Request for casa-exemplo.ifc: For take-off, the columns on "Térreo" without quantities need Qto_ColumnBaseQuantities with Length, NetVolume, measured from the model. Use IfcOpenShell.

First a look at what the model holds.

```python
import ifcopenshell
import ifcopenshell.util.element
import ifcopenshell.util.unit

model = ifcopenshell.open("casa-exemplo.ifc")
print(model.schema)
for unit_type in ("LENGTHUNIT", "AREAUNIT", "VOLUMEUNIT"):
    print(unit_type, ifcopenshell.util.unit.calculate_unit_scale(model, unit_type))
storey = next(s for s in model.by_type("IfcBuildingStorey") if s.Name == "Térreo")
columns = [e for e in ifcopenshell.util.element.get_decomposition(storey) if e.is_a("IfcColumn")]
for e in sorted(columns, key=lambda e: e.id()):
    print(e.id(), e.is_a(), e.Name, list(ifcopenshell.util.element.get_psets(e, qtos_only=True)), sep=" | ")
```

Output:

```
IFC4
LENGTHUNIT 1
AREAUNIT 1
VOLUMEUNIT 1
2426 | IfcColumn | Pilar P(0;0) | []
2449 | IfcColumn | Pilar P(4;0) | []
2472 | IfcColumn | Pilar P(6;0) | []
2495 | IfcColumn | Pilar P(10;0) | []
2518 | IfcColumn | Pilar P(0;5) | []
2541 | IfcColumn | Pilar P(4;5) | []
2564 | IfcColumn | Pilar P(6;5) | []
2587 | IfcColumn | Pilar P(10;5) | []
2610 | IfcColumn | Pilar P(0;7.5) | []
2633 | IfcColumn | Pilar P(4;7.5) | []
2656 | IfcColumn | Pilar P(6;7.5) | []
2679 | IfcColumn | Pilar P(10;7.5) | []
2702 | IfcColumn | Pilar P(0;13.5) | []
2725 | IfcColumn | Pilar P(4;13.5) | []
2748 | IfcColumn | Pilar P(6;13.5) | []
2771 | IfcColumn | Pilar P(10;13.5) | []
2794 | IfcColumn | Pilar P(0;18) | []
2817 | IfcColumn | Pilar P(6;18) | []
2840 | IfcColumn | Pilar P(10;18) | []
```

```python
import ifcopenshell
import ifcopenshell.api.pset
import ifcopenshell.geom
import ifcopenshell.util.element
import ifcopenshell.util.shape
import ifcopenshell.util.unit

model = ifcopenshell.open("casa-exemplo.ifc")
unit_scale = ifcopenshell.util.unit.calculate_unit_scale(model)
volume_scale = ifcopenshell.util.unit.calculate_unit_scale(model, "VOLUMEUNIT")
settings = ifcopenshell.geom.settings()

storey = next(s for s in model.by_type("IfcBuildingStorey") if s.Name == "Térreo")
columns = [e for e in ifcopenshell.util.element.get_decomposition(storey) if e.is_a("IfcColumn")]

for e in sorted(columns, key=lambda e: e.id()):
    if ifcopenshell.util.element.get_psets(e, qtos_only=True, should_inherit=False):
        continue
    # Geometry comes back in metres, in the element's own axes.
    shape = ifcopenshell.geom.create_shape(settings, e)
    values = {
        "Length": ifcopenshell.util.shape.get_z(shape.geometry) / unit_scale,
        "NetVolume": ifcopenshell.util.shape.get_volume(shape.geometry) / volume_scale,
    }
    qto = ifcopenshell.api.pset.add_qto(model, product=e, name="Qto_ColumnBaseQuantities")
    ifcopenshell.api.pset.edit_qto(model, qto=qto, properties=values)
    print(e.id(), {k: round(v, 3) for k, v in values.items()})

model.write("casa-exemplo_v2.ifc")
```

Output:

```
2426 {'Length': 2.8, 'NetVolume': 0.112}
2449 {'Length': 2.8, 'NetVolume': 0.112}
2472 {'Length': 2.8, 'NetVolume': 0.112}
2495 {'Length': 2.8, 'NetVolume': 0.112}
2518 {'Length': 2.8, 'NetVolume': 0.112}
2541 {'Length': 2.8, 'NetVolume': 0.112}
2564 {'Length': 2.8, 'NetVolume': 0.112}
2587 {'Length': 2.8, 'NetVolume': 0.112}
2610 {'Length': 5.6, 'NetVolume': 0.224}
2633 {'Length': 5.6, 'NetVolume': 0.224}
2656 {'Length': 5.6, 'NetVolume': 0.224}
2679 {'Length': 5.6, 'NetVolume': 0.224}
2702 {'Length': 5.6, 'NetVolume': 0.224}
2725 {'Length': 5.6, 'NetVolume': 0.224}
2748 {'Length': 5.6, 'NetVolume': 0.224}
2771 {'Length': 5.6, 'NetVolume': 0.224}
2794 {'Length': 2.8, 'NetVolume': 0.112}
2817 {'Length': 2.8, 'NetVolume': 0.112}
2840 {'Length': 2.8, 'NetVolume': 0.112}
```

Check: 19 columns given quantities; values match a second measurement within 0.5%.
